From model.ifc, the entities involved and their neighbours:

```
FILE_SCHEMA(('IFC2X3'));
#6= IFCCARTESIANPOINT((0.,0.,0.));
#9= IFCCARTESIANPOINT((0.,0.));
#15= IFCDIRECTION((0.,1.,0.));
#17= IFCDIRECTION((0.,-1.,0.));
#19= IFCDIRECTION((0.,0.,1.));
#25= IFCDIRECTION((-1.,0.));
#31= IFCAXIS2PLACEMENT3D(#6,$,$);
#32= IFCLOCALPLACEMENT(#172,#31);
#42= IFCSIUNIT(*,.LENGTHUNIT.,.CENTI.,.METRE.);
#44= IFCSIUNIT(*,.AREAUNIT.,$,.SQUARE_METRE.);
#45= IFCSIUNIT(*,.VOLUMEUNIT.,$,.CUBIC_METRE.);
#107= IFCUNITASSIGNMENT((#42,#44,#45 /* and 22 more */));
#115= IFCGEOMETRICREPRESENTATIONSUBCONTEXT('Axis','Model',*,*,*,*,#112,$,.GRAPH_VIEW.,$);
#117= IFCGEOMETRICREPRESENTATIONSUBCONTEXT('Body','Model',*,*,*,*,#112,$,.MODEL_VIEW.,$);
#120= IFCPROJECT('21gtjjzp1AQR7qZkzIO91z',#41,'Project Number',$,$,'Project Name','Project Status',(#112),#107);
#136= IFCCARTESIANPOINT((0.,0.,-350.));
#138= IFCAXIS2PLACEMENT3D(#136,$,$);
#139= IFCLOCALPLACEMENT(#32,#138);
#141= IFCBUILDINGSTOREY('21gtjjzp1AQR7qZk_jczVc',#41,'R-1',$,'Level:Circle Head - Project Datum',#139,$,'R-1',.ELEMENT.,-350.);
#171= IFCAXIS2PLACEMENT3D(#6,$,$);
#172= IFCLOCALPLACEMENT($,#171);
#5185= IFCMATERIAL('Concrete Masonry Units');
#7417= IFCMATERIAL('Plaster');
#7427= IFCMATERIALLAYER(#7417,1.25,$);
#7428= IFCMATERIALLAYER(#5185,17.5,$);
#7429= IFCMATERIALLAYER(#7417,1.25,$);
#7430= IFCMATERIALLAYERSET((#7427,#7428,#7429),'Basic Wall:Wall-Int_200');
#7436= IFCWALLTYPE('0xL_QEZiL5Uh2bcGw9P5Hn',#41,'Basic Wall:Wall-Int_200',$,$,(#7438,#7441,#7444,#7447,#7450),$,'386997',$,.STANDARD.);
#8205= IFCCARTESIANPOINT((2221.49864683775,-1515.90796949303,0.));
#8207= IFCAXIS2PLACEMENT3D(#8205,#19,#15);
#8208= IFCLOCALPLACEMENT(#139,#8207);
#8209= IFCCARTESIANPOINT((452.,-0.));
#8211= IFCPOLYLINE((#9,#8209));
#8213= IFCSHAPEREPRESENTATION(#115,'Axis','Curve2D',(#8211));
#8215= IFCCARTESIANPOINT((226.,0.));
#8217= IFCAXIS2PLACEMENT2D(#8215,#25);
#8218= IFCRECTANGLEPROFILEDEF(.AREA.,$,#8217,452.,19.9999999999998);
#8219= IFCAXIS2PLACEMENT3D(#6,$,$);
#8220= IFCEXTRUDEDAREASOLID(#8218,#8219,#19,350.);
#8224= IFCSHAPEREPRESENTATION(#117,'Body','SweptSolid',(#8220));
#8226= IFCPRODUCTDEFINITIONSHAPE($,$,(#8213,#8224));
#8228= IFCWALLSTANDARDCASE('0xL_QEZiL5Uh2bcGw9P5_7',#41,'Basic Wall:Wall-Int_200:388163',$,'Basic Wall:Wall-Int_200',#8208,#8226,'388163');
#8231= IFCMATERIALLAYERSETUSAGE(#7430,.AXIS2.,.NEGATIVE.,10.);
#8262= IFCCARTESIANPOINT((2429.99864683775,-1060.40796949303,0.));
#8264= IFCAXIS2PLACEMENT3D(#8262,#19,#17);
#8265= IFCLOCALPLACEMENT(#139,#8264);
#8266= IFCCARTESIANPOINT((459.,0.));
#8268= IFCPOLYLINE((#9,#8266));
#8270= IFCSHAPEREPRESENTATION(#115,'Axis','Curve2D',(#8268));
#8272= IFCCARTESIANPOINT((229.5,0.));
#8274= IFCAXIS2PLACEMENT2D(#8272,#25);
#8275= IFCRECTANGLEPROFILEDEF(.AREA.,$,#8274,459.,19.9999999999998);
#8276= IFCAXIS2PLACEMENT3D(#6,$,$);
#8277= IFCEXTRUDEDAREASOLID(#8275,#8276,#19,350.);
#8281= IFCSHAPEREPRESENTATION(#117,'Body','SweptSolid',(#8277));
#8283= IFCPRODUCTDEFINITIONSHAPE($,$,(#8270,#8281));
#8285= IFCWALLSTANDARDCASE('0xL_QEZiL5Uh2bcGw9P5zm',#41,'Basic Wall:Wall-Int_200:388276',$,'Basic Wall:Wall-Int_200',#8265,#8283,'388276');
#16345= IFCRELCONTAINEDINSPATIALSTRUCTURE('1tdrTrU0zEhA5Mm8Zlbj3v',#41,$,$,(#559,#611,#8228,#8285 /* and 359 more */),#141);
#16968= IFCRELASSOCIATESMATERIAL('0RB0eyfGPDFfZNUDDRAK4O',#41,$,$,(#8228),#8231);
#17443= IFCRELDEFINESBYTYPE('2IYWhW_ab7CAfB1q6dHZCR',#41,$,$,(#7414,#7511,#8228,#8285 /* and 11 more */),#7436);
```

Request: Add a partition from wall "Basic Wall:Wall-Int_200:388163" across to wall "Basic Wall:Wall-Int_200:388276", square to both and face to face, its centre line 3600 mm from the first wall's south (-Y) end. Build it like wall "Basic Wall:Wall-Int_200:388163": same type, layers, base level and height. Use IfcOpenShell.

```python
import numpy as np
import ifcopenshell
import ifcopenshell.api.geometry
import ifcopenshell.api.material
import ifcopenshell.api.pset
import ifcopenshell.api.root
import ifcopenshell.api.spatial
import ifcopenshell.api.type
import ifcopenshell.geom
import ifcopenshell.util.element
import ifcopenshell.util.placement
import ifcopenshell.util.representation
import ifcopenshell.util.shape
import ifcopenshell.util.unit

model = ifcopenshell.open("model.ifc")
unit_scale = ifcopenshell.util.unit.calculate_unit_scale(model)
settings = ifcopenshell.geom.settings()
settings.set("use-world-coords", True)

start_wall = model.by_guid("0xL_QEZiL5Uh2bcGw9P5_7")
end_wall = model.by_guid("0xL_QEZiL5Uh2bcGw9P5zm")
like = model.by_guid("0xL_QEZiL5Uh2bcGw9P5_7")
matrix = ifcopenshell.util.placement.get_local_placement(start_wall.ObjectPlacement)
matrix[:3, 3] *= unit_scale


def extent(element):
    """Bounding box in the first wall's axes, in metres."""
    shape = ifcopenshell.geom.create_shape(settings, element)
    points = (ifcopenshell.util.shape.get_vertices(shape.geometry) - matrix[:3, 3]) @ matrix[:3, :3]
    return points.min(axis=0), points.max(axis=0)


y_start = extent(start_wall)[0][1]
y_end = extent(end_wall)[1][1]
like_min, like_max = extent(like)
length, height = float(abs(y_end - y_start)), float(like_max[2] - like_min[2])
layer_set = ifcopenshell.util.element.get_material(like, should_skip_usage=True)
thickness = sum(layer.LayerThickness for layer in layer_set.MaterialLayers) * unit_scale

wall = ifcopenshell.api.root.create_entity(model, ifc_class="IfcWallStandardCase", name="New partition")
storey = ifcopenshell.util.element.get_container(like)
ifcopenshell.api.spatial.assign_container(model, products=[wall], relating_structure=storey)
ifcopenshell.api.type.assign_type(
    model, related_objects=[wall], relating_type=ifcopenshell.util.element.get_type(like), should_map_representations=False
)
rel = ifcopenshell.api.material.assign_material(
    model, products=[wall], type="IfcMaterialLayerSetUsage", material=layer_set
)
rel.RelatingMaterial.OffsetFromReferenceLine = -thickness / 2 / unit_scale
pset = ifcopenshell.api.pset.add_pset(model, product=wall, name="Pset_WallCommon")
ifcopenshell.api.pset.edit_pset(model, pset=pset, properties={"IsExternal": False, "LoadBearing": False})

# The axis runs down the middle of the wall.
axis = ifcopenshell.api.geometry.add_axis_representation(
    model, context=ifcopenshell.util.representation.get_context(model, "Model", "Axis"), axis=[(0.0, 0.0), (length, 0.0)]
)
body = ifcopenshell.api.geometry.add_wall_representation(
    model,
    context=ifcopenshell.util.representation.get_context(model, "Model", "Body", "MODEL_VIEW"),
    length=length,
    height=height,
    thickness=thickness,
    offset=-thickness / 2,
)
for representation in (axis, body):
    ifcopenshell.api.geometry.assign_representation(model, product=wall, representation=representation)

placement = matrix @ ifcopenshell.util.placement.rotation(-90, "Z")
placement[:, 3] = matrix @ np.array([extent(start_wall)[0][0] + 3.6, y_start, like_min[2], 1.0])
ifcopenshell.api.geometry.edit_object_placement(model, product=wall, matrix=placement)

print(f"partition {length:.3f} m long, {height:.3f} m high, {thickness:.3f} m thick")

model.write("model_updated.ifc")
```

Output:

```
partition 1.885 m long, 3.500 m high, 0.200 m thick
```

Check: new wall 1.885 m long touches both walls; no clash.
